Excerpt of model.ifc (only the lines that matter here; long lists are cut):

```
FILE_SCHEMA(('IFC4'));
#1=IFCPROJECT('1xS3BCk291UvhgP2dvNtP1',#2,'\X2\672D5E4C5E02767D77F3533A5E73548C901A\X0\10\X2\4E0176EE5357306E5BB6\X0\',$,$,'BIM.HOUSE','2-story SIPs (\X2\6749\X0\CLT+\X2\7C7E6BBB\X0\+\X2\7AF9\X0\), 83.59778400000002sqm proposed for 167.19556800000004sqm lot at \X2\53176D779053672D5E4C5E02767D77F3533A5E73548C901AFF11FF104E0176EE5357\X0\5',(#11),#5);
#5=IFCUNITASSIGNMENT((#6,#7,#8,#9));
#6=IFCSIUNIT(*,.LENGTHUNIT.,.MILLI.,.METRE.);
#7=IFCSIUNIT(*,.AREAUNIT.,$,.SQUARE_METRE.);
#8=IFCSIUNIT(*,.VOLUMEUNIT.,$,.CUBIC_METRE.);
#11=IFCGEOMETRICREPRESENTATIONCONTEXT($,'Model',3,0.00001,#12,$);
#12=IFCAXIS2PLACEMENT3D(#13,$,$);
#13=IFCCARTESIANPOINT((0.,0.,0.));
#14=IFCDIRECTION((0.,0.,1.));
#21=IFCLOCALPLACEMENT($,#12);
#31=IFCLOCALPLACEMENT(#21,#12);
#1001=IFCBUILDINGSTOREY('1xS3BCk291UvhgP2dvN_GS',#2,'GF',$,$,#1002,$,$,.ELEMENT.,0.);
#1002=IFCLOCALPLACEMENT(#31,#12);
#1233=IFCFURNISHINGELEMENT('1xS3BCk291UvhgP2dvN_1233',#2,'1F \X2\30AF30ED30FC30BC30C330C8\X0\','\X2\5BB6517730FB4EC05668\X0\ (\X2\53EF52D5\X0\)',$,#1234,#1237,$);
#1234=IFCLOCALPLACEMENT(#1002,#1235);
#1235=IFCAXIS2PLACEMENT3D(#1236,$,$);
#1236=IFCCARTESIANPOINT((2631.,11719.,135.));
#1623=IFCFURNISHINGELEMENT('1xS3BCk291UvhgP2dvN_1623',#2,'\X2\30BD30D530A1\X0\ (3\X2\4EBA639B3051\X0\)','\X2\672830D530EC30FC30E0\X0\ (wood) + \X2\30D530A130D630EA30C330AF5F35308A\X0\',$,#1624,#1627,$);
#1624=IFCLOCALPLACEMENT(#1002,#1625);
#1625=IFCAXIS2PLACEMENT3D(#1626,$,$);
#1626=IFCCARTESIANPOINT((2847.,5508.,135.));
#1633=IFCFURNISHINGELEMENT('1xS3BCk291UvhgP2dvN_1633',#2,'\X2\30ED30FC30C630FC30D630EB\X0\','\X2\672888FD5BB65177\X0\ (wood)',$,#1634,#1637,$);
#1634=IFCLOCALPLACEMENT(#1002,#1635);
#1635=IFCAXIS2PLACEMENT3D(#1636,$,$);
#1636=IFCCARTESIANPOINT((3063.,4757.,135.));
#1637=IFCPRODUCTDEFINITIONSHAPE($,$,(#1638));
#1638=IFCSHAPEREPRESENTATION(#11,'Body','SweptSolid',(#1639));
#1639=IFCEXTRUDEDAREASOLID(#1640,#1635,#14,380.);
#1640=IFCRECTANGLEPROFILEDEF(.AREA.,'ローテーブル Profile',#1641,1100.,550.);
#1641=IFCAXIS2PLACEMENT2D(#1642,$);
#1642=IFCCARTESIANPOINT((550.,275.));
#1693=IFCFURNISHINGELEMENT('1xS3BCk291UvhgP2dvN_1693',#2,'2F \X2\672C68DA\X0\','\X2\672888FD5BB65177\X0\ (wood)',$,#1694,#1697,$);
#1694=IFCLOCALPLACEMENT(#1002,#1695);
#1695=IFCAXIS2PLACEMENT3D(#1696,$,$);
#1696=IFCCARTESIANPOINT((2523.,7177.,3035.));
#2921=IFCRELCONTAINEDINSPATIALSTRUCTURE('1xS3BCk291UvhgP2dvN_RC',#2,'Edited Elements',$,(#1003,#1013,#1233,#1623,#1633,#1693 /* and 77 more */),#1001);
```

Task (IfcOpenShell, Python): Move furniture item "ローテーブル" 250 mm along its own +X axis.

```python
import ifcopenshell
import ifcopenshell.api.geometry
import ifcopenshell.util.placement
import ifcopenshell.util.unit

model = ifcopenshell.open("model.ifc")
unit_scale = ifcopenshell.util.unit.calculate_unit_scale(model)

item = model.by_id(1633)
matrix = ifcopenshell.util.placement.get_local_placement(item.ObjectPlacement)
matrix[:3, 3] += matrix[:3, 0] * 0.25 / unit_scale
ifcopenshell.api.geometry.edit_object_placement(model, product=item, matrix=matrix, is_si=False)

print(ifcopenshell.util.placement.get_local_placement(item.ObjectPlacement).round(3) + 0.0)

model.write("model_edited.ifc")
```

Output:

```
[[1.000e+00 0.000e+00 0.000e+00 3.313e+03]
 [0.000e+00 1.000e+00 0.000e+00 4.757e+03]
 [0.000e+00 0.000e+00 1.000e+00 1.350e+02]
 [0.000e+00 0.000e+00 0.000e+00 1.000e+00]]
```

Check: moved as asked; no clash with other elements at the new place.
